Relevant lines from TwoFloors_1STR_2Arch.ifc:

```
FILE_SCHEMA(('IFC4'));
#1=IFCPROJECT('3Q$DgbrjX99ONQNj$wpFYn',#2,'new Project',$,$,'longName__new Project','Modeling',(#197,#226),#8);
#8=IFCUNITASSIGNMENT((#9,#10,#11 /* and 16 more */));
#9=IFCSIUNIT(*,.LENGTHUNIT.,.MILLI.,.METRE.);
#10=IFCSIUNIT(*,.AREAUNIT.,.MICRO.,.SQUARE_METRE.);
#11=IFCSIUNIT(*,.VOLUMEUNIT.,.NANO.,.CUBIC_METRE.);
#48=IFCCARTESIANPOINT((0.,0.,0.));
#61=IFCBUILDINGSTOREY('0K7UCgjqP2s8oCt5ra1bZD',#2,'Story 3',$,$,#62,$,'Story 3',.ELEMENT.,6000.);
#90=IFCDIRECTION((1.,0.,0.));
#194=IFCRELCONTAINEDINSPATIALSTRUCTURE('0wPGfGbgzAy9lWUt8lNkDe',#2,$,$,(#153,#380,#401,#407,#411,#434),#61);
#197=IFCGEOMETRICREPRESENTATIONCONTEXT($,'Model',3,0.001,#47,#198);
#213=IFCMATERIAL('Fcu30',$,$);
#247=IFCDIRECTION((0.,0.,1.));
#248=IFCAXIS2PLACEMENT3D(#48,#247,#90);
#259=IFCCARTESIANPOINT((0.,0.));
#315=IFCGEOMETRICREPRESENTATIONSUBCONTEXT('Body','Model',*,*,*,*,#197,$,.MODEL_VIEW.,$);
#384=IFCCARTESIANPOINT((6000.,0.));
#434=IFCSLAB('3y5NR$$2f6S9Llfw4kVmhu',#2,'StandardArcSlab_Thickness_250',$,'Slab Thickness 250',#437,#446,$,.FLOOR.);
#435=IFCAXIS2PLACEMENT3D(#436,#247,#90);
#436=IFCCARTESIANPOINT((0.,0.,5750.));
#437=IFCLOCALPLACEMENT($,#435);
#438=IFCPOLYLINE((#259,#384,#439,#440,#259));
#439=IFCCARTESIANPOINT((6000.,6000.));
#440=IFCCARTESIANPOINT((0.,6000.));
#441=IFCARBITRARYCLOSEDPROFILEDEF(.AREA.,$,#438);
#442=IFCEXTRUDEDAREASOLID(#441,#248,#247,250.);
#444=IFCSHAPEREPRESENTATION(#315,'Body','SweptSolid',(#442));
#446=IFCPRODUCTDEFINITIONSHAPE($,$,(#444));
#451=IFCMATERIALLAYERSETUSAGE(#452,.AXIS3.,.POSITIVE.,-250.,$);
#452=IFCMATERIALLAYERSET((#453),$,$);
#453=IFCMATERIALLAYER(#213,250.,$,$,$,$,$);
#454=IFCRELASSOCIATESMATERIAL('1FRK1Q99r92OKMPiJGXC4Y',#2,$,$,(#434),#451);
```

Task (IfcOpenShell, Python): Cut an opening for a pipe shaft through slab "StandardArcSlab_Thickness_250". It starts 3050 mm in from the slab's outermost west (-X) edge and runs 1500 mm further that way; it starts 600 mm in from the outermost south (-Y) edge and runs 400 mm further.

```python
import numpy as np
import ifcopenshell
import ifcopenshell.api.feature
import ifcopenshell.api.geometry
import ifcopenshell.api.root
import ifcopenshell.geom
import ifcopenshell.util.placement
import ifcopenshell.util.representation
import ifcopenshell.util.shape
import ifcopenshell.util.unit

model = ifcopenshell.open("TwoFloors_1STR_2Arch.ifc")
unit_scale = ifcopenshell.util.unit.calculate_unit_scale(model)
settings = ifcopenshell.geom.settings()


def volume(element):
    """Net volume in cubic metres, openings subtracted."""
    shape = ifcopenshell.geom.create_shape(settings, element)
    return ifcopenshell.util.shape.get_volume(shape.geometry)


slab = model.by_guid("3y5NR$$2f6S9Llfw4kVmhu")
before = volume(slab)

# Extent in the slab's own axes, in metres. The edges named are its -X and -Y sides.
slab_shape = ifcopenshell.geom.create_shape(settings, slab)
vertices = ifcopenshell.util.shape.get_vertices(slab_shape.geometry)
x_min, y_min, bottom = vertices.min(axis=0)
top = vertices[:, 2].max()

opening = ifcopenshell.api.root.create_entity(model, ifc_class="IfcOpeningElement", name="Pipe shaft opening", predefined_type="OPENING")
context = ifcopenshell.util.representation.get_context(model, "Model", "Body", "MODEL_VIEW")
width, depth = 1.5, 0.4
outline = [(0.0, 0.0), (width, 0.0), (width, depth), (0.0, depth), (0.0, 0.0)]
# Overshoot both faces by 50 mm so the cut is clean.
shape = ifcopenshell.api.geometry.add_slab_representation(
    model, context=context, depth=top - bottom + 0.1, polyline=outline
)
ifcopenshell.api.geometry.assign_representation(model, product=opening, representation=shape)

matrix = ifcopenshell.util.placement.get_local_placement(slab.ObjectPlacement)
matrix[:, 3] = matrix @ np.append(np.array([x_min + 3.05, y_min + 0.6, bottom - 0.05]) / unit_scale, 1.0)
ifcopenshell.api.geometry.edit_object_placement(model, product=opening, matrix=matrix, is_si=False)
ifcopenshell.api.feature.add_feature(model, feature=opening, element=slab)

after = volume(slab)

print(f"slab volume {before:.3f} -> {after:.3f} m3")

model.write("TwoFloors_1STR_2Arch_v2.ifc")
```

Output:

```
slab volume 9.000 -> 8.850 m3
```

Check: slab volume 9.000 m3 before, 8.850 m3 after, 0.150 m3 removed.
